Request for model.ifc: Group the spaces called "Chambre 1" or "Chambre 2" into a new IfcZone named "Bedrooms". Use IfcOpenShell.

First a look at what the model holds.

```python
import ifcopenshell

model = ifcopenshell.open("model.ifc")
print(model.schema)
seen = {}
for space in model.by_type("IfcSpace"):
    seen[space.LongName] = seen.get(space.LongName, 0) + 1
for name, count in sorted(seen.items(), key=str):
    print(count, "x", name)
print("zones:", [z.Name for z in model.by_type("IfcZone")][:20])
```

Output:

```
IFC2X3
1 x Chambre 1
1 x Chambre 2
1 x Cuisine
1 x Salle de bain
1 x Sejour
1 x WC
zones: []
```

```python
import ifcopenshell
import ifcopenshell.api.group
import ifcopenshell.api.root

model = ifcopenshell.open("model.ifc")

names = {"Chambre 1", "Chambre 2"}
spaces = [s for s in model.by_type("IfcSpace") if s.LongName in names]

zone = ifcopenshell.api.root.create_entity(model, ifc_class="IfcZone", name="Bedrooms")
ifcopenshell.api.group.assign_group(model, products=spaces, group=zone)
print(len(spaces), "spaces in", zone.Name)

model.write("model_rev.ifc")
```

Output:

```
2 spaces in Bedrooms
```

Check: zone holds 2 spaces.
